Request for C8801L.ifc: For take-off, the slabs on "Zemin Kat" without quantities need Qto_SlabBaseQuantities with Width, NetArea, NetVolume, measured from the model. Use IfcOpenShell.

First a look at what the model holds.

```python
import ifcopenshell
import ifcopenshell.util.element
import ifcopenshell.util.unit

model = ifcopenshell.open("C8801L.ifc")
print(model.schema)
for unit_type in ("LENGTHUNIT", "AREAUNIT", "VOLUMEUNIT"):
    print(unit_type, ifcopenshell.util.unit.calculate_unit_scale(model, unit_type))
storey = next(s for s in model.by_type("IfcBuildingStorey") if s.Name == "Zemin Kat")
slabs = [e for e in ifcopenshell.util.element.get_decomposition(storey) if e.is_a("IfcSlab")]
for e in sorted(slabs, key=lambda e: e.id()):
    print(e.id(), e.is_a(), e.Name, list(ifcopenshell.util.element.get_psets(e, qtos_only=True)), sep=" | ")
```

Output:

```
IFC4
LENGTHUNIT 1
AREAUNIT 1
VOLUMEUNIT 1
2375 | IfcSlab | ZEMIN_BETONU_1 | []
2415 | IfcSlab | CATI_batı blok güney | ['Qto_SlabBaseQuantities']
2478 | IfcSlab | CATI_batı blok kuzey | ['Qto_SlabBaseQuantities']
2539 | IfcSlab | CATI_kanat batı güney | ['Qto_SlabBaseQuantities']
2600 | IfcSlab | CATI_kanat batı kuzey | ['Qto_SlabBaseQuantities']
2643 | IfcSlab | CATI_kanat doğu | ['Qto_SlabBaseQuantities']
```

```python
import ifcopenshell
import ifcopenshell.api.pset
import ifcopenshell.geom
import ifcopenshell.util.element
import ifcopenshell.util.shape
import ifcopenshell.util.unit

model = ifcopenshell.open("C8801L.ifc")
unit_scale = ifcopenshell.util.unit.calculate_unit_scale(model)
area_scale = ifcopenshell.util.unit.calculate_unit_scale(model, "AREAUNIT")
volume_scale = ifcopenshell.util.unit.calculate_unit_scale(model, "VOLUMEUNIT")
settings = ifcopenshell.geom.settings()

storey = next(s for s in model.by_type("IfcBuildingStorey") if s.Name == "Zemin Kat")
slabs = [e for e in ifcopenshell.util.element.get_decomposition(storey) if e.is_a("IfcSlab")]

for e in sorted(slabs, key=lambda e: e.id()):
    if ifcopenshell.util.element.get_psets(e, qtos_only=True, should_inherit=False):
        continue
    # Geometry comes back in metres, in the element's own axes.
    shape = ifcopenshell.geom.create_shape(settings, e)
    values = {
        "Width": ifcopenshell.util.shape.get_z(shape.geometry) / unit_scale,
        "NetArea": ifcopenshell.util.shape.get_footprint_area(shape.geometry) / area_scale,
        "NetVolume": ifcopenshell.util.shape.get_volume(shape.geometry) / volume_scale,
    }
    qto = ifcopenshell.api.pset.add_qto(model, product=e, name="Qto_SlabBaseQuantities")
    ifcopenshell.api.pset.edit_qto(model, qto=qto, properties=values)
    print(e.id(), {k: round(v, 3) for k, v in values.items()})

model.write("C8801L_rev.ifc")
```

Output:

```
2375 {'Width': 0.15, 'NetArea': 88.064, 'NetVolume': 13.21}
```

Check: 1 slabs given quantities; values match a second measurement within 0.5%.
